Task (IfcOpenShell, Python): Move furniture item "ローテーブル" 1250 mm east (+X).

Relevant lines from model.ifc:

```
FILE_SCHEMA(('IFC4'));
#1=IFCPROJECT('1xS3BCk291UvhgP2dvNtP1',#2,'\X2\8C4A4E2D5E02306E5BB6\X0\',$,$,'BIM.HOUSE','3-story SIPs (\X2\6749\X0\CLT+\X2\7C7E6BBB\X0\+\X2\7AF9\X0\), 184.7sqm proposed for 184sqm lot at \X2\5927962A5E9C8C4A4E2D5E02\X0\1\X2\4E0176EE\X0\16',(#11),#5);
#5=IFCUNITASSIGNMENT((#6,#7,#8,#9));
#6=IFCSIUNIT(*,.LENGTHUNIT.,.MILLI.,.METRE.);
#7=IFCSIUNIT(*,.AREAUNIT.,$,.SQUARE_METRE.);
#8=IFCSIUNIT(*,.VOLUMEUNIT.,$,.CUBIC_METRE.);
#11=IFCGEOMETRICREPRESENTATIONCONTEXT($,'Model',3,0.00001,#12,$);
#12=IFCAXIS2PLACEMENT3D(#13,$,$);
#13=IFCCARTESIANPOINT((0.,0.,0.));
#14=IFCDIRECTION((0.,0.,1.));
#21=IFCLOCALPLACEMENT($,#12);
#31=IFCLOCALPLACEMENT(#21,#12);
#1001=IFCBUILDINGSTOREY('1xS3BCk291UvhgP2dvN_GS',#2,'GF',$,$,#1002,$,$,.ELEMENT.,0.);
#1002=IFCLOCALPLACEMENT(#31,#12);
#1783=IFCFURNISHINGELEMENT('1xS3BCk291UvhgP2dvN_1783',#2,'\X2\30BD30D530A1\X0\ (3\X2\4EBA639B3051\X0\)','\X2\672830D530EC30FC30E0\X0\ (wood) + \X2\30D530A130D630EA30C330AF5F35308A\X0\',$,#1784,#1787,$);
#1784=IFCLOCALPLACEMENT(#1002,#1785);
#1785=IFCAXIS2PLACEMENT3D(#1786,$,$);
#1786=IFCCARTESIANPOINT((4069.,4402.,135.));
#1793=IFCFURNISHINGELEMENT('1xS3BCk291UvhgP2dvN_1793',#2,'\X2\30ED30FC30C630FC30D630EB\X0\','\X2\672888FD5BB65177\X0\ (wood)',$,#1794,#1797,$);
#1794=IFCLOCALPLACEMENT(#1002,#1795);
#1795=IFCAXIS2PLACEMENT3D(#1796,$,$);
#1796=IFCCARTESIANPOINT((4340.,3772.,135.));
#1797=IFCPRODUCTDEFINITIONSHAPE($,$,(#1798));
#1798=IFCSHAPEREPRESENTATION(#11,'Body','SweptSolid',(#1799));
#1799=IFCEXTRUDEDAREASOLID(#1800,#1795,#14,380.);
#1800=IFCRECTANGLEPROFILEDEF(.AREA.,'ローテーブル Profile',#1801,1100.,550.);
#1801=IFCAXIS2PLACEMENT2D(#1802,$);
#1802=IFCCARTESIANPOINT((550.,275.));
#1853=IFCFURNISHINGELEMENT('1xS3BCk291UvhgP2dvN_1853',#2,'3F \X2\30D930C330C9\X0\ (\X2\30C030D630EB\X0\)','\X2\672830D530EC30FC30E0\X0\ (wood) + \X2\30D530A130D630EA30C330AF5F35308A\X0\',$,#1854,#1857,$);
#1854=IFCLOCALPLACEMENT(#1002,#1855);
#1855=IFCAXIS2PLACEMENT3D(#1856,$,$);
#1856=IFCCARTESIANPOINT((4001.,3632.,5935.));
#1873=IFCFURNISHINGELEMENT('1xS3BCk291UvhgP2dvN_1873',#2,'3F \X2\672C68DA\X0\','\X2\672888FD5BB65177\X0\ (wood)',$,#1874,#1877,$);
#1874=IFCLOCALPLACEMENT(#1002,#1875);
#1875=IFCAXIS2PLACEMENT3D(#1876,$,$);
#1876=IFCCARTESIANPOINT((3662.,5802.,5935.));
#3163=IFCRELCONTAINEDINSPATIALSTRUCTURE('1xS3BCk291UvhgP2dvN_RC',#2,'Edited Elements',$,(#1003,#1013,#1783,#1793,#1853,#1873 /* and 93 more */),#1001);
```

```python
import ifcopenshell
import ifcopenshell.api.geometry
import ifcopenshell.util.placement
import ifcopenshell.util.unit

model = ifcopenshell.open("model.ifc")
unit_scale = ifcopenshell.util.unit.calculate_unit_scale(model)

item = model.by_guid("1xS3BCk291UvhgP2dvN_1793")
matrix = ifcopenshell.util.placement.get_local_placement(item.ObjectPlacement)
matrix[0, 3] += 1.25 / unit_scale
ifcopenshell.api.geometry.edit_object_placement(model, product=item, matrix=matrix, is_si=False)

print(ifcopenshell.util.placement.get_local_placement(item.ObjectPlacement).round(3) + 0.0)

model.write("model-out.ifc")
```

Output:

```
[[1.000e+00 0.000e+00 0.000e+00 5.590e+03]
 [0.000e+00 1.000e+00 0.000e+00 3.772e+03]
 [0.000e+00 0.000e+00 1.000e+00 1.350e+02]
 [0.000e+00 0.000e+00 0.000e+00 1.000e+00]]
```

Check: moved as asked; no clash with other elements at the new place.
